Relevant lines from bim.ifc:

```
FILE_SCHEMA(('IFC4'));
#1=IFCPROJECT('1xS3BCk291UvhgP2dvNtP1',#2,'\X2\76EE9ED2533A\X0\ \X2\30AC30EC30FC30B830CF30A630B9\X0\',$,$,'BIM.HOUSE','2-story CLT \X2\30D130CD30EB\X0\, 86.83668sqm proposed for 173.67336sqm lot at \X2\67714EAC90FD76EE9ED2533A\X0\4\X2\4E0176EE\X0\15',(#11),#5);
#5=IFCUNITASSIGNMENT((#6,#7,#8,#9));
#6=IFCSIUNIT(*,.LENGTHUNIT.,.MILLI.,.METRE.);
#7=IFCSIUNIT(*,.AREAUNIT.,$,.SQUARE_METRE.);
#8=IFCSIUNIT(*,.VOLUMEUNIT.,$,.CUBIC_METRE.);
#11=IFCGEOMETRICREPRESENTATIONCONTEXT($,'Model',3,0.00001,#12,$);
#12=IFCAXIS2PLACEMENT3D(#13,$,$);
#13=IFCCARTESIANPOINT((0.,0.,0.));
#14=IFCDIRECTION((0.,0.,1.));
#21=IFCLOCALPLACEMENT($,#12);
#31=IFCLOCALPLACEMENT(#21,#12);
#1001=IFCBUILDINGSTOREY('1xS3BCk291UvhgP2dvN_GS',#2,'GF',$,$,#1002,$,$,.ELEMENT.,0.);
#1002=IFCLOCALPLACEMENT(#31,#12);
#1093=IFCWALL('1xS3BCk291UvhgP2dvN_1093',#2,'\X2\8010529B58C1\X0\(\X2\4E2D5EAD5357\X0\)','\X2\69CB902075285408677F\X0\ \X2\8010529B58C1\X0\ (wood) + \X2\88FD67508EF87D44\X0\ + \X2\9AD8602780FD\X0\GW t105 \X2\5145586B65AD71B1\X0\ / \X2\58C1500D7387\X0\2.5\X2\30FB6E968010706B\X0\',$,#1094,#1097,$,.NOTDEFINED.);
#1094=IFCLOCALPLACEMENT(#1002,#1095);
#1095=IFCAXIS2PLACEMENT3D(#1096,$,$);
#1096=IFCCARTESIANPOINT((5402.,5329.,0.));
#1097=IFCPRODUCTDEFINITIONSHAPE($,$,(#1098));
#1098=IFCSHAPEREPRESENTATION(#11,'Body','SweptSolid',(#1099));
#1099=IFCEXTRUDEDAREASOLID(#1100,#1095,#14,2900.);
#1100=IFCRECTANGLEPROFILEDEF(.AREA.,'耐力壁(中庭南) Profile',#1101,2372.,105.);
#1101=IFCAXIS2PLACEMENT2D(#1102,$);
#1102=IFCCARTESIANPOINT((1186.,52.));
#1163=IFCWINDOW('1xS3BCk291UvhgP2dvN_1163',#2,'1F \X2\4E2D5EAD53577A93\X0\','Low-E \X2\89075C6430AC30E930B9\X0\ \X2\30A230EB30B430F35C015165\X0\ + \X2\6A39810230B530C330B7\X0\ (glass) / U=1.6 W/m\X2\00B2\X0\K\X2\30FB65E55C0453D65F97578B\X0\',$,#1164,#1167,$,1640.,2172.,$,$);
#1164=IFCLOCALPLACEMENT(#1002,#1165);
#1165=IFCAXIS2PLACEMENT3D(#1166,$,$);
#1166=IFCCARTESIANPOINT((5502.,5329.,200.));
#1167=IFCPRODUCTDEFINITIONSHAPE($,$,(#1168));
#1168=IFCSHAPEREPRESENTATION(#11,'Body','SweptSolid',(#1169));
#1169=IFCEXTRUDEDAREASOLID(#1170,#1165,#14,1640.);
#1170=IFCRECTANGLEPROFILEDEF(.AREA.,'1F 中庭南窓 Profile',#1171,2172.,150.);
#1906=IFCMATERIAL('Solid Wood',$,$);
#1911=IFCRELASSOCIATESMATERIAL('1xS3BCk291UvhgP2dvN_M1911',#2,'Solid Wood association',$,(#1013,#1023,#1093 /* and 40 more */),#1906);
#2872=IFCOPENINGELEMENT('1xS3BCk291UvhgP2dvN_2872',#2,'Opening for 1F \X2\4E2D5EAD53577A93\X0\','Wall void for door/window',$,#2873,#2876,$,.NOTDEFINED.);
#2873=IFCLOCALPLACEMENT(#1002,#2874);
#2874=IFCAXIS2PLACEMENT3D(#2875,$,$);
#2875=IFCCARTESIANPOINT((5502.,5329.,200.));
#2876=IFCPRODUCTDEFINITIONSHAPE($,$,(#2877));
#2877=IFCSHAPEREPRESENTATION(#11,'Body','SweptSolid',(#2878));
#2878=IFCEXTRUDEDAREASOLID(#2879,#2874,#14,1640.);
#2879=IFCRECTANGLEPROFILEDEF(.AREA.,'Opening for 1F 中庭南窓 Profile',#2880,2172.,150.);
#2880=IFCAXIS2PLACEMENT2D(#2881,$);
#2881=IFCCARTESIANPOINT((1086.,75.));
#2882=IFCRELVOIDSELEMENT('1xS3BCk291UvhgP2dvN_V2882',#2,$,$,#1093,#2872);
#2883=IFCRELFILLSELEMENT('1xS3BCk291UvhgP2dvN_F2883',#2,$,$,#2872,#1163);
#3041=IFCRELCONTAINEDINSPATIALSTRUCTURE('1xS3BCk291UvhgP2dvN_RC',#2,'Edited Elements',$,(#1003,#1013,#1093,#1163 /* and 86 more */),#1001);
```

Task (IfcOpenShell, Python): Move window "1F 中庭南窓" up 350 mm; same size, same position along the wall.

```python
import numpy as np
import ifcopenshell
import ifcopenshell.api.geometry
import ifcopenshell.util.placement
import ifcopenshell.util.unit

model = ifcopenshell.open("bim.ifc")
unit_scale = ifcopenshell.util.unit.calculate_unit_scale(model)

window = model.by_guid("1xS3BCk291UvhgP2dvN_1163")
opening = window.FillsVoids[0].RelatingOpeningElement
dz = 350.0

shift = np.array([0.0, 0.0, dz])
# The window is not placed relative to its opening, so move both.
for product in (opening, window):
    matrix = ifcopenshell.util.placement.get_local_placement(product.ObjectPlacement)
    matrix[:3, 3] += shift
    ifcopenshell.api.geometry.edit_object_placement(model, product=product, matrix=matrix, is_si=False)

print(f"moved by {dz * unit_scale:+.3f} m")

model.write("bim_rev.ifc")
```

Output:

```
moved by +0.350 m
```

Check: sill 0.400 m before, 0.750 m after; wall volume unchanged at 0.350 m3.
